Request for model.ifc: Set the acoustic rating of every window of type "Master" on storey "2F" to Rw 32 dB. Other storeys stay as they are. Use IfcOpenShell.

First a look at what the model holds.

```python
import ifcopenshell
import ifcopenshell.util.element

model = ifcopenshell.open("model.ifc")
print(model.schema)
storey = next(s for s in model.by_type("IfcBuildingStorey") if s.Name == "2F")
windows = [e for e in ifcopenshell.util.element.get_decomposition(storey) if e.is_a("IfcWindow")]
seen = {}
for e in windows:
    element_type = ifcopenshell.util.element.get_type(e)
    key = (element_type.Name if element_type != e and element_type else None, ifcopenshell.util.element.get_pset(e, "Pset_WindowCommon", "AcousticRating"))
    seen[key] = seen.get(key, 0) + 1
for (name, value), count in sorted(seen.items(), key=str):
    print(count, "x", name, "|", value)
```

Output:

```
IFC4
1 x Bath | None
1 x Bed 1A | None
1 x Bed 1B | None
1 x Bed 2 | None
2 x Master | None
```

```python
import ifcopenshell
import ifcopenshell.api.pset
import ifcopenshell.util.element

model = ifcopenshell.open("model.ifc")

storey = next(s for s in model.by_type("IfcBuildingStorey") if s.Name == "2F")
windows = [e for e in ifcopenshell.util.element.get_decomposition(storey) if e.is_a("IfcWindow")]

count = 0
for e in windows:
    element_type = ifcopenshell.util.element.get_type(e)
    if element_type in (None, e) or element_type.Name != "Master":
        continue
    # add_pset returns the element's existing set when there is one.
    pset = ifcopenshell.api.pset.add_pset(model, product=e, name="Pset_WindowCommon")
    ifcopenshell.api.pset.edit_pset(model, pset=pset, properties={"AcousticRating": "Rw 32 dB"})
    count += 1

print(count, "windows updated")

model.write("model_v2.ifc")
```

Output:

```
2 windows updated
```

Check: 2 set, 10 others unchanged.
